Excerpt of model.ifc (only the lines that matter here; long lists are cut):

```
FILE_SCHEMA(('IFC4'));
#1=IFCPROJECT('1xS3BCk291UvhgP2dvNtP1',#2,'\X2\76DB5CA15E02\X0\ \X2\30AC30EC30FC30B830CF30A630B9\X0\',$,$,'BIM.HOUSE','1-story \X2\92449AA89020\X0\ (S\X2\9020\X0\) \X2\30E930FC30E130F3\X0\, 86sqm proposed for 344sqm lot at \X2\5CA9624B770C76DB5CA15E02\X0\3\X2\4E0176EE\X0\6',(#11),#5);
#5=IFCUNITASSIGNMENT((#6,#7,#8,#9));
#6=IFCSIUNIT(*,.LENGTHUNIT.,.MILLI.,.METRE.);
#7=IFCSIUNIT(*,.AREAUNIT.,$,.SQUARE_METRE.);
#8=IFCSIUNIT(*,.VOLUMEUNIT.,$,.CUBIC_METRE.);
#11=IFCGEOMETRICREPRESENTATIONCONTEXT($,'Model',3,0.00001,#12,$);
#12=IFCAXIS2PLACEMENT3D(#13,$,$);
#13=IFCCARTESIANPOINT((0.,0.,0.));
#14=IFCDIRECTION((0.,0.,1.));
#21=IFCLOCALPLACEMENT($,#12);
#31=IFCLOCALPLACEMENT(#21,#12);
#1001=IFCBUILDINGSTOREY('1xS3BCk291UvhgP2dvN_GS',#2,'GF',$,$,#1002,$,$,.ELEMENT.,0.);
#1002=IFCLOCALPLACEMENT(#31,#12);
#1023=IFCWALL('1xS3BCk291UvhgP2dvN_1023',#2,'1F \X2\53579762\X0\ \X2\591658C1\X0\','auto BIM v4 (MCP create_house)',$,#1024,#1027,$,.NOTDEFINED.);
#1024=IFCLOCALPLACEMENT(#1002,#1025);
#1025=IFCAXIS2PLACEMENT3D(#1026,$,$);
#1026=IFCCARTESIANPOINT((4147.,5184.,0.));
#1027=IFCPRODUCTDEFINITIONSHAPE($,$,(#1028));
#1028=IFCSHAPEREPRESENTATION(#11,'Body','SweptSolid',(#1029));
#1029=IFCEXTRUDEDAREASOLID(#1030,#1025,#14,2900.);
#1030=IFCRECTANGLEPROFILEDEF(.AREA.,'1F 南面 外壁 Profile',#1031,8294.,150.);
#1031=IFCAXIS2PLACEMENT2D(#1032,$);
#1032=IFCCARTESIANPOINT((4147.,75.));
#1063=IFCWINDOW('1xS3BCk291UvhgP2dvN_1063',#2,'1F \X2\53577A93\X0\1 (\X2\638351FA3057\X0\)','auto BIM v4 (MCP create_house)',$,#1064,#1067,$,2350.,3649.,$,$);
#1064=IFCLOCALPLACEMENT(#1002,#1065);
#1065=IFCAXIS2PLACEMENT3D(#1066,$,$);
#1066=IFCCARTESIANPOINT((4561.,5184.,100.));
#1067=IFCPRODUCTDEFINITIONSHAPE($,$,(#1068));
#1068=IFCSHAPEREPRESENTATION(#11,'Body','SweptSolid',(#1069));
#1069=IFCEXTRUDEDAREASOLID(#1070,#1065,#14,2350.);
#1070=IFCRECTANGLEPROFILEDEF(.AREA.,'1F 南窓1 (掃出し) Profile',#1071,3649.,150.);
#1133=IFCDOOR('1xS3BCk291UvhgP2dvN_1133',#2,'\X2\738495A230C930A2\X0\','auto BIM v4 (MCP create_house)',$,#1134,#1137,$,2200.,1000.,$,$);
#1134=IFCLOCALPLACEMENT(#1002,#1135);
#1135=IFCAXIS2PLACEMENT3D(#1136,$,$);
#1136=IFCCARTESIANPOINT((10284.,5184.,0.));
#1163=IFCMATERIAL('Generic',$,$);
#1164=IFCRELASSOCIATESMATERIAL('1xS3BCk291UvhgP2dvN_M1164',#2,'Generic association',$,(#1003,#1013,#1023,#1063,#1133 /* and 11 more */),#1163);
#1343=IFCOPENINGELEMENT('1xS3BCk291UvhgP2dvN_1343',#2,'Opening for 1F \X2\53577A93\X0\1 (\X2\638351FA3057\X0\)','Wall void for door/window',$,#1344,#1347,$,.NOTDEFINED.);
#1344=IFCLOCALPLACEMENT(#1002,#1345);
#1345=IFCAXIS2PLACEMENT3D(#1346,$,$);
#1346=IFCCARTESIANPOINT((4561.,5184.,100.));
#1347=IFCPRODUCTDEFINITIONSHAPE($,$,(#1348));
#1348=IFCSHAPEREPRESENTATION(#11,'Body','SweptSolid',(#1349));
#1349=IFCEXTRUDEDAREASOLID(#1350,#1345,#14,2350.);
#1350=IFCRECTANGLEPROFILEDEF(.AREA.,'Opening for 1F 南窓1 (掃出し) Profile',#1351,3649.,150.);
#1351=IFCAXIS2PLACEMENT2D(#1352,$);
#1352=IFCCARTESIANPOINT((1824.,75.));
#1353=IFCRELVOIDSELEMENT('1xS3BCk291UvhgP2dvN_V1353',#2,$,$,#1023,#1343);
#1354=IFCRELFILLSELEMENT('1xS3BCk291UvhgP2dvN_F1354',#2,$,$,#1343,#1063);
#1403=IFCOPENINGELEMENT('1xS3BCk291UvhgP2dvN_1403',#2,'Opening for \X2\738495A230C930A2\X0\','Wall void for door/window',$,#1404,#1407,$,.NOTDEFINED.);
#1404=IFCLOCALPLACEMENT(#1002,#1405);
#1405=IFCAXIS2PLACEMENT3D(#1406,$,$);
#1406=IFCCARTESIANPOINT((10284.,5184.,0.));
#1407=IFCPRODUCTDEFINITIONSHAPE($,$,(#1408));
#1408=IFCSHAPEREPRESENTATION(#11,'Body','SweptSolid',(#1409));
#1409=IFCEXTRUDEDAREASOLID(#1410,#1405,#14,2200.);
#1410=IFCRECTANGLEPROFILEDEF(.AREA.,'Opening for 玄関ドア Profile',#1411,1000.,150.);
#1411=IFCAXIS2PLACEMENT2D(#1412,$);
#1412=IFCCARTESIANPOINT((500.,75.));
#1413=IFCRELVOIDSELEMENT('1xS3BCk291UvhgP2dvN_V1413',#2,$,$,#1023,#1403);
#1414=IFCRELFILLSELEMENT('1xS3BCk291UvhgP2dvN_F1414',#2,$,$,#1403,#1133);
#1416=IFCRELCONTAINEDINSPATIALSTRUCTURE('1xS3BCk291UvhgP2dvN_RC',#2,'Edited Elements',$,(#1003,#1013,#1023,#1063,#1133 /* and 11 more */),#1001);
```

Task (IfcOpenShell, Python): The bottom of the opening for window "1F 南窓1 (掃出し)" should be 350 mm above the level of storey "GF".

```python
import numpy as np
import ifcopenshell
import ifcopenshell.api.geometry
import ifcopenshell.geom
import ifcopenshell.util.element
import ifcopenshell.util.placement
import ifcopenshell.util.shape
import ifcopenshell.util.unit

model = ifcopenshell.open("model.ifc")
unit_scale = ifcopenshell.util.unit.calculate_unit_scale(model)

window = model.by_guid("1xS3BCk291UvhgP2dvN_1063")
opening = window.FillsVoids[0].RelatingOpeningElement
storey = ifcopenshell.util.element.get_container(window, ifc_class="IfcBuildingStorey")
level = ifcopenshell.util.placement.get_local_placement(storey.ObjectPlacement)[2, 3]

# The opening's origin need not be at the sill, so measure its lowest point.
shape = ifcopenshell.geom.create_shape(ifcopenshell.geom.settings(), opening)
bottom = ifcopenshell.util.shape.get_shape_bottom_elevation(shape, shape.geometry) / unit_scale
dz = level + 350.0 - bottom

shift = np.array([0.0, 0.0, dz])
# The window is not placed relative to its opening, so move both.
for product in (opening, window):
    matrix = ifcopenshell.util.placement.get_local_placement(product.ObjectPlacement)
    matrix[:3, 3] += shift
    ifcopenshell.api.geometry.edit_object_placement(model, product=product, matrix=matrix, is_si=False)

print(f"moved by {dz * unit_scale:+.3f} m")

model.write("model_v2.ifc")
```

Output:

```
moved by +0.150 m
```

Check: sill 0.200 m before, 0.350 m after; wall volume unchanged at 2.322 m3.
